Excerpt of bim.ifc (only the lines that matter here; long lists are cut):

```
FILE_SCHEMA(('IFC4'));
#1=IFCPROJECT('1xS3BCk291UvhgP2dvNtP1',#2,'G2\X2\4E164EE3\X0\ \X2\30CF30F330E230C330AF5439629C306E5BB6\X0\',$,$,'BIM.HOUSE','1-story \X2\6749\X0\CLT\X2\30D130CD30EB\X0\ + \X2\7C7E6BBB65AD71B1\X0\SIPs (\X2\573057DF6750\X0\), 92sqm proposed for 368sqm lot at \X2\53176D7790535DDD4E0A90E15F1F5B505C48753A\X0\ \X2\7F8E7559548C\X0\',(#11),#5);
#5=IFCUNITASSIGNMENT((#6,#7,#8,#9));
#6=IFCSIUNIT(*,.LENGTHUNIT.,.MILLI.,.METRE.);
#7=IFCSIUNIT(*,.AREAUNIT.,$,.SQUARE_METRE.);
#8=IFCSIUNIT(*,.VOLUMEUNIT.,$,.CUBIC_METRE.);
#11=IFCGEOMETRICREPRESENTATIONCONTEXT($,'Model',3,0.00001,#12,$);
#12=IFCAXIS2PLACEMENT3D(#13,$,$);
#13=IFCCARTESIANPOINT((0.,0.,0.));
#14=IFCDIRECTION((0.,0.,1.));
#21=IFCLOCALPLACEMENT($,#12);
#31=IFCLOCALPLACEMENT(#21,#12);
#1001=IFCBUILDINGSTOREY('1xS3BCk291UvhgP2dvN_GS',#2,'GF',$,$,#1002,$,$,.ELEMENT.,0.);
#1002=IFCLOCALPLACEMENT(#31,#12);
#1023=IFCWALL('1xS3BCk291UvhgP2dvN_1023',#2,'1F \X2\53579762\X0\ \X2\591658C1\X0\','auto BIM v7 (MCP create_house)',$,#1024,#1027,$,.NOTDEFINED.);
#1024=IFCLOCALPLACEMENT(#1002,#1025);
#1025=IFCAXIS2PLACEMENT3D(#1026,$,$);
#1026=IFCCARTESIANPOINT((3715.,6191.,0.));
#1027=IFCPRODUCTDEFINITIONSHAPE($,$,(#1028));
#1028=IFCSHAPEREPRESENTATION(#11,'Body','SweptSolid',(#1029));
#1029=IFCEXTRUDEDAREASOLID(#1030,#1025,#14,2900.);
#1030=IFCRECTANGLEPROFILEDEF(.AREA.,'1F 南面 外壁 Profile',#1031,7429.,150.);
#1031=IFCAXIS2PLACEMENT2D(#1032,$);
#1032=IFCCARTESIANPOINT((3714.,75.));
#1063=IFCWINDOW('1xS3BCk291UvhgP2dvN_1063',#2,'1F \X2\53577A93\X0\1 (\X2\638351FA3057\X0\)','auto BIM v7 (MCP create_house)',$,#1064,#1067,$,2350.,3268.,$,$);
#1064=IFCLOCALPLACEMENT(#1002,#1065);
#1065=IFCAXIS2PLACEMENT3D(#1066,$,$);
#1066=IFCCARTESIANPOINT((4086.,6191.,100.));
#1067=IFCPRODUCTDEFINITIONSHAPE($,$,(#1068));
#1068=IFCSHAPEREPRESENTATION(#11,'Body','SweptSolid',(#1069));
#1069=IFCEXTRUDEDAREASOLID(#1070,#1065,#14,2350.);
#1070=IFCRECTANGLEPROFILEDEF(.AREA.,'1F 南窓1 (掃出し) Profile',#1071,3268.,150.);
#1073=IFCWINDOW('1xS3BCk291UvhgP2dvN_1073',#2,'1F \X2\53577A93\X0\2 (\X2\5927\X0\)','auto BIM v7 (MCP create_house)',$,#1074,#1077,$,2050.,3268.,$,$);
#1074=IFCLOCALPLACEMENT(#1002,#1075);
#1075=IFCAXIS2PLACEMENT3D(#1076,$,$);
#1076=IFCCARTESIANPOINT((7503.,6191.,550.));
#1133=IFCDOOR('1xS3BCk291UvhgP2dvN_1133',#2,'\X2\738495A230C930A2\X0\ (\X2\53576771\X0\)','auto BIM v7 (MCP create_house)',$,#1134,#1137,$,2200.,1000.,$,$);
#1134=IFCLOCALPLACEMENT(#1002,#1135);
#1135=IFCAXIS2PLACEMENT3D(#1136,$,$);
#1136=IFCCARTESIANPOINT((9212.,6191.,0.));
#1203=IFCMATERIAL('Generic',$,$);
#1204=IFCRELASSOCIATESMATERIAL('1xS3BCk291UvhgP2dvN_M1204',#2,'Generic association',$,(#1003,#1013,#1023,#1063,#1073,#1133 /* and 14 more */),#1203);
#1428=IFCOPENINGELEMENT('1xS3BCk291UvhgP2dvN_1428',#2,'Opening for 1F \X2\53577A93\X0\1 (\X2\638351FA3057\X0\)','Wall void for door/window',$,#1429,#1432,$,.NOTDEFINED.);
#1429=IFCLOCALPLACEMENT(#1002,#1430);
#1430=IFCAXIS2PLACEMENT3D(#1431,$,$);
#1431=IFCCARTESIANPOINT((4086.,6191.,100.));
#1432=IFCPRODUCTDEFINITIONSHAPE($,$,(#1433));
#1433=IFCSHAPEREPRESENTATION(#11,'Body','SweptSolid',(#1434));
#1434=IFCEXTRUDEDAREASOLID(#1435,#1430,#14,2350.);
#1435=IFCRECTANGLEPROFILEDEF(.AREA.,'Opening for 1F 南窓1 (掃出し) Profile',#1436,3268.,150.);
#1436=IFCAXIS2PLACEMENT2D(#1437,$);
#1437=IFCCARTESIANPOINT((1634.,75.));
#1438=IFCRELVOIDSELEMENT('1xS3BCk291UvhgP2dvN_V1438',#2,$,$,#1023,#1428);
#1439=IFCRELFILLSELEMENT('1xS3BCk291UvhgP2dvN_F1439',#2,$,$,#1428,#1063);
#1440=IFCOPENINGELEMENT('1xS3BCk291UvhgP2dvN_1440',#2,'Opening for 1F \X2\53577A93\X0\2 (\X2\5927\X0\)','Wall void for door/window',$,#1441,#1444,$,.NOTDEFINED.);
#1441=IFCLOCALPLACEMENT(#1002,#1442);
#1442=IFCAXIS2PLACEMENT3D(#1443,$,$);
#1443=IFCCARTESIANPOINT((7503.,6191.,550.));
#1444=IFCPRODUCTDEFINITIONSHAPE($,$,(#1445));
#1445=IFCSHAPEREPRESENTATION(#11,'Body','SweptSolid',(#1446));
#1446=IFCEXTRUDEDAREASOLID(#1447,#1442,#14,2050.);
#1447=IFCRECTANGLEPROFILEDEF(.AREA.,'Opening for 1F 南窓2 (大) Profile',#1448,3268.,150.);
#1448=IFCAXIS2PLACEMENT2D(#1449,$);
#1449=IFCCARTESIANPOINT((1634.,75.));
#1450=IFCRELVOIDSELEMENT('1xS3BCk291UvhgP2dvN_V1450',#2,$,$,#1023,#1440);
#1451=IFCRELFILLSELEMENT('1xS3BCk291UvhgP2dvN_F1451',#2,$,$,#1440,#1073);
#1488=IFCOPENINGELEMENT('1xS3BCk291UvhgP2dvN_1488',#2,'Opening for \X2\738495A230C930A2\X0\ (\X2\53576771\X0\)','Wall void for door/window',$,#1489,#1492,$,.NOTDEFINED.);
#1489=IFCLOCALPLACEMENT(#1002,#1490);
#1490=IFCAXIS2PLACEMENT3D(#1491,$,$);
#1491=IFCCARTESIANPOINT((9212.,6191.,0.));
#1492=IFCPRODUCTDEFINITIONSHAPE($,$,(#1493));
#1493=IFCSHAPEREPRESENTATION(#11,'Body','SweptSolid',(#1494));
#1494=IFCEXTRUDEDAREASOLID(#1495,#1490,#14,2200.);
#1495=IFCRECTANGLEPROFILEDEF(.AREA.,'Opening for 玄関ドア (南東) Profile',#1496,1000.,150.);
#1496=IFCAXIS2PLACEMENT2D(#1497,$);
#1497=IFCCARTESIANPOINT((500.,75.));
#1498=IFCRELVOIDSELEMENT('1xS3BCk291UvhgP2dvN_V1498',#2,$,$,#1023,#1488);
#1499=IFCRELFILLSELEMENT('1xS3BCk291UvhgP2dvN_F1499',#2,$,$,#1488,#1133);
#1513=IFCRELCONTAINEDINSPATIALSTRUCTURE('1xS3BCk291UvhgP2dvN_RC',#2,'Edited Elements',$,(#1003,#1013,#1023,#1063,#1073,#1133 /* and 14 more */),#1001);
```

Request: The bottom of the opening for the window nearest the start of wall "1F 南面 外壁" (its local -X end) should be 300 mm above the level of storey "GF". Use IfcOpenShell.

```python
import numpy as np
import ifcopenshell
import ifcopenshell.api.geometry
import ifcopenshell.geom
import ifcopenshell.util.element
import ifcopenshell.util.placement
import ifcopenshell.util.shape
import ifcopenshell.util.unit

model = ifcopenshell.open("bim.ifc")
unit_scale = ifcopenshell.util.unit.calculate_unit_scale(model)

window = model.by_guid("1xS3BCk291UvhgP2dvN_1063")
opening = window.FillsVoids[0].RelatingOpeningElement
storey = ifcopenshell.util.element.get_container(window, ifc_class="IfcBuildingStorey")
level = ifcopenshell.util.placement.get_local_placement(storey.ObjectPlacement)[2, 3]

# The opening's origin need not be at the sill, so measure its lowest point.
shape = ifcopenshell.geom.create_shape(ifcopenshell.geom.settings(), opening)
bottom = ifcopenshell.util.shape.get_shape_bottom_elevation(shape, shape.geometry) / unit_scale
dz = level + 0.3 / unit_scale - bottom

shift = np.array([0.0, 0.0, dz])
# The window is not placed relative to its opening, so move both.
for product in (opening, window):
    matrix = ifcopenshell.util.placement.get_local_placement(product.ObjectPlacement)
    matrix[:3, 3] += shift
    ifcopenshell.api.geometry.edit_object_placement(model, product=product, matrix=matrix, is_si=False)

print(f"moved by {dz * unit_scale:+.3f} m")

model.write("bim_v2.ifc")
```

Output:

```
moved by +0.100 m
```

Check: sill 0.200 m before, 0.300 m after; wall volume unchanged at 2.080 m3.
